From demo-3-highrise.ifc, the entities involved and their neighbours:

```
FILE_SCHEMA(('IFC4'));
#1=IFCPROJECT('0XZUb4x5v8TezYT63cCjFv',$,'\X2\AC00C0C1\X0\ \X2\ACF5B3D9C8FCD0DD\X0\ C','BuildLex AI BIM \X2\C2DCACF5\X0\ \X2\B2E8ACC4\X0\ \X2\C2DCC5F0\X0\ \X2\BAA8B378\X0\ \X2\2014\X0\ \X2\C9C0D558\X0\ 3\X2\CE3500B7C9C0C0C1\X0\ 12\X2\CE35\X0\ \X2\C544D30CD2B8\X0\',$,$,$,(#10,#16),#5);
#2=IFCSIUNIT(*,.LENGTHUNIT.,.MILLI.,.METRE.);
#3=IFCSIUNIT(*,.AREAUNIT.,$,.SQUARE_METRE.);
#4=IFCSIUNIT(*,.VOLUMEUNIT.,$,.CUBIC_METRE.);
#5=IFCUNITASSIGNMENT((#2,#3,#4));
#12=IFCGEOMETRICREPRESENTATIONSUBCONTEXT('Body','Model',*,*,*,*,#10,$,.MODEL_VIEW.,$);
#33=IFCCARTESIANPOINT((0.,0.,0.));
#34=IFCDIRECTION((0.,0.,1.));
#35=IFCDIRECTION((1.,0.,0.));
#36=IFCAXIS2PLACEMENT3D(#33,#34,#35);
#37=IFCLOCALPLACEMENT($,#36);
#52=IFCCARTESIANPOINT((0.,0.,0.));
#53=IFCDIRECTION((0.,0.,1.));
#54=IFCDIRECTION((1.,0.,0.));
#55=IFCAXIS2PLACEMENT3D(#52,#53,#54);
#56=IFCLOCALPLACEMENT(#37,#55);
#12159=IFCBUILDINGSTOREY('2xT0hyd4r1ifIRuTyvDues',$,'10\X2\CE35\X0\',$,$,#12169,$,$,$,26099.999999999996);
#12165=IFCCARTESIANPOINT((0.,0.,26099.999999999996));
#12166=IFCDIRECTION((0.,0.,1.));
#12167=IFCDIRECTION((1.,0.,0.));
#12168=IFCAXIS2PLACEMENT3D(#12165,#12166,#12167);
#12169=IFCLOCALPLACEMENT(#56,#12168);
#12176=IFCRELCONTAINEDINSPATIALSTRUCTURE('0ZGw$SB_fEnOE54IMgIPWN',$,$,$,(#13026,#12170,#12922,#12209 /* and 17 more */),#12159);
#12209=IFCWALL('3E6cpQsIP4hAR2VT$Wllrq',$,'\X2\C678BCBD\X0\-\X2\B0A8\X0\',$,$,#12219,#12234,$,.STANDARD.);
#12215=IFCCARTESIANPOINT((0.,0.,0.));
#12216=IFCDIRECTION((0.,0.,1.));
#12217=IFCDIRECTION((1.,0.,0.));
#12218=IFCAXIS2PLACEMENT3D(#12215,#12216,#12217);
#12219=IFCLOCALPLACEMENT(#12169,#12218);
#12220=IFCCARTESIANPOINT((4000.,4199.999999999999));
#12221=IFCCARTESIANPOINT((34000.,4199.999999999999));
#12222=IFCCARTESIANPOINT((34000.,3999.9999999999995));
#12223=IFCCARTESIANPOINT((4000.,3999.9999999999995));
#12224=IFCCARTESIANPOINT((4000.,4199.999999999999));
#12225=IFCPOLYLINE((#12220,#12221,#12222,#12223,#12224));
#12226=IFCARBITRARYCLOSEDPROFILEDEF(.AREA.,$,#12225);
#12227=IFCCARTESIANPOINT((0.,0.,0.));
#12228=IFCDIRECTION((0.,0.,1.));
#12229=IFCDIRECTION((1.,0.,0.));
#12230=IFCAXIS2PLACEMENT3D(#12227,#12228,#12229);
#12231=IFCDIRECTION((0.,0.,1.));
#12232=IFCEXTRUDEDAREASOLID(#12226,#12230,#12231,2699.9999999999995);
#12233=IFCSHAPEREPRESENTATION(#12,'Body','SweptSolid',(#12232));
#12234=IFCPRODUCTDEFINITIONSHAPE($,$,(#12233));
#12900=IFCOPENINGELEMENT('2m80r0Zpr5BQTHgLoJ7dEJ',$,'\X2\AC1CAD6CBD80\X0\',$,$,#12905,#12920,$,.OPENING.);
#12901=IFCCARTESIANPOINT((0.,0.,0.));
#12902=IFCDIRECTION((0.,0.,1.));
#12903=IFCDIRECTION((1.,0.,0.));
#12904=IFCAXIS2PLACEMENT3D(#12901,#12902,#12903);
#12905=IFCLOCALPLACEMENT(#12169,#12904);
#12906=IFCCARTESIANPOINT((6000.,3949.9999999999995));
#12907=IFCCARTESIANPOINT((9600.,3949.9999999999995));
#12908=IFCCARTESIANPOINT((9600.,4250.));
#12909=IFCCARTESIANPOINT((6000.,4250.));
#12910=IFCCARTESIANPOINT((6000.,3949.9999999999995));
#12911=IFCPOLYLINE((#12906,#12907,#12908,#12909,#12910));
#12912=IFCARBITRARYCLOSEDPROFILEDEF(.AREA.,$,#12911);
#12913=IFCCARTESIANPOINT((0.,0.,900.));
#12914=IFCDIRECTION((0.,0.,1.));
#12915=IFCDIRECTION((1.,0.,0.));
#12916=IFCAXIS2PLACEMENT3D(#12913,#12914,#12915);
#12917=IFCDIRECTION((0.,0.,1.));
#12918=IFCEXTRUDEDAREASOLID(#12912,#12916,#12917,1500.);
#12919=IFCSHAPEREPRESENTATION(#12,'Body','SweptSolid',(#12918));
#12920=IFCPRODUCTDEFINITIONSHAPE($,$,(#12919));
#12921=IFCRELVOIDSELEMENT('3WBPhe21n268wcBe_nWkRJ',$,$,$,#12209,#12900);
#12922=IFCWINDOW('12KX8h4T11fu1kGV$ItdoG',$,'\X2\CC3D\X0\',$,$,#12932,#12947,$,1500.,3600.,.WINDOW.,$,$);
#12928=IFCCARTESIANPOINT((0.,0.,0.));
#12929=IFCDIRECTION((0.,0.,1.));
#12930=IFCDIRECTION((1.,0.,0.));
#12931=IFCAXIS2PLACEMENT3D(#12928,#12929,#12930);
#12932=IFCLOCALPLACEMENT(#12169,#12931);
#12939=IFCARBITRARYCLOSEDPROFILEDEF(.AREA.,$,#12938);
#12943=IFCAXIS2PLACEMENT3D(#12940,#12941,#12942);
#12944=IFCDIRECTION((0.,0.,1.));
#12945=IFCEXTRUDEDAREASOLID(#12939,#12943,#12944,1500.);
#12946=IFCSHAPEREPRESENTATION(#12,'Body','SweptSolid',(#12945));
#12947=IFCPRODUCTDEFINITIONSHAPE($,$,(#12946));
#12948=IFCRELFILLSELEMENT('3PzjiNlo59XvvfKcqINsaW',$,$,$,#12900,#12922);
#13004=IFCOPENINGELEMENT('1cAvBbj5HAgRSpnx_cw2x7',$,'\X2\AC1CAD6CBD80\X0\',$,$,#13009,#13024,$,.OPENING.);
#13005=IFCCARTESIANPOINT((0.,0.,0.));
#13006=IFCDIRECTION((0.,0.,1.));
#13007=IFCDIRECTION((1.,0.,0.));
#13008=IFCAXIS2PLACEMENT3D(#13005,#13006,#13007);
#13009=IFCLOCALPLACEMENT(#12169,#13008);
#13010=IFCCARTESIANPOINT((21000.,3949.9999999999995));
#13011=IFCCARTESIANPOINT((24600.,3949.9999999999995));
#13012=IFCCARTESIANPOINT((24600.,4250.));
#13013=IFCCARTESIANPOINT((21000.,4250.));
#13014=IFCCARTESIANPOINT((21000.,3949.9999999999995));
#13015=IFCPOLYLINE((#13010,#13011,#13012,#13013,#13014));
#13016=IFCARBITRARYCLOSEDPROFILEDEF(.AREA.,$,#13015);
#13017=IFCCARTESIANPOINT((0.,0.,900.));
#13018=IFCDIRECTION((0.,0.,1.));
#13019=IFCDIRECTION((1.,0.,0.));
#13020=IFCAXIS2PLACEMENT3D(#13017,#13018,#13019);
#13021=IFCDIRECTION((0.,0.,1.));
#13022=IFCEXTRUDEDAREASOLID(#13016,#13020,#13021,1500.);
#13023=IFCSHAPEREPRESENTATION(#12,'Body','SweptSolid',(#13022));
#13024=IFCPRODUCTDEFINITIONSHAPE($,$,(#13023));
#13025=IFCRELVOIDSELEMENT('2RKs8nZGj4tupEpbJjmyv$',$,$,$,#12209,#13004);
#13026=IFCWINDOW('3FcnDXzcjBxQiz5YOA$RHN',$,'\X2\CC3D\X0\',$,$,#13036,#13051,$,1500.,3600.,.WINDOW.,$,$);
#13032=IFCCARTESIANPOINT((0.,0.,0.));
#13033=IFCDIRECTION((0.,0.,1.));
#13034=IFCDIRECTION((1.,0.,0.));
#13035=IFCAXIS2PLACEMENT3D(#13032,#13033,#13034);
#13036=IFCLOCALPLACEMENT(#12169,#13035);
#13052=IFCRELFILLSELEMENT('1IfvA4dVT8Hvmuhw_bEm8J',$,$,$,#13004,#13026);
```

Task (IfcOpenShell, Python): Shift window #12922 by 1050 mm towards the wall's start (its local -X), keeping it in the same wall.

```python
import ifcopenshell
import ifcopenshell.api.geometry
import ifcopenshell.util.placement
import ifcopenshell.util.unit

model = ifcopenshell.open("demo-3-highrise.ifc")
unit_scale = ifcopenshell.util.unit.calculate_unit_scale(model)

window = model.by_id(12922)
opening = window.FillsVoids[0].RelatingOpeningElement
wall = opening.VoidsElements[0].RelatingBuildingElement

wall_matrix = ifcopenshell.util.placement.get_local_placement(wall.ObjectPlacement)
shift = wall_matrix[:3, 0] * -1.05 / unit_scale
before = ifcopenshell.util.placement.get_local_placement(window.ObjectPlacement)[:3, 3].copy()

# The window is not placed relative to its opening, so move both.
for product in (opening, window):
    matrix = ifcopenshell.util.placement.get_local_placement(product.ObjectPlacement)
    matrix[:3, 3] += shift
    ifcopenshell.api.geometry.edit_object_placement(model, product=product, matrix=matrix, is_si=False)

after = ifcopenshell.util.placement.get_local_placement(window.ObjectPlacement)[:3, 3]
print("window moved by", (after - before).round(3) + 0.0)

model.write("demo-3-highrise-out.ifc")
```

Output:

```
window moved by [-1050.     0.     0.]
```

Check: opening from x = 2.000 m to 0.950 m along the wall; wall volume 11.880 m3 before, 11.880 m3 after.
